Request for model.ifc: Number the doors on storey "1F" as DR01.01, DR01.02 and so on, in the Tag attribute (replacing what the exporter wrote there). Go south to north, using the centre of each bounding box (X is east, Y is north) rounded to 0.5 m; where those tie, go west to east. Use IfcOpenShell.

First a look at what the model holds.

```python
import ifcopenshell
import ifcopenshell.util.element
import ifcopenshell.util.placement

model = ifcopenshell.open("model.ifc")
print(model.schema)
storey = next(s for s in model.by_type("IfcBuildingStorey") if s.Name == "1F")
doors = [e for e in ifcopenshell.util.element.get_decomposition(storey) if e.is_a("IfcDoor")]
for e in sorted(doors, key=lambda e: e.id()):
    origin = ifcopenshell.util.placement.get_local_placement(e.ObjectPlacement)[:3, 3]
    print(e.id(), e.Tag, e.Name, origin.round(2) + 0.0, sep=" | ")
```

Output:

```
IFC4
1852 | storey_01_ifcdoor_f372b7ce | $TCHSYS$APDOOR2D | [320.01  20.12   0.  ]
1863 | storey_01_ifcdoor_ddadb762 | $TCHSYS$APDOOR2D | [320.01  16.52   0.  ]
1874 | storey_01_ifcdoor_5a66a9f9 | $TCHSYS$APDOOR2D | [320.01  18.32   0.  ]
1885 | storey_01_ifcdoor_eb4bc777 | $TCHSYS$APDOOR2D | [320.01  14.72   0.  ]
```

```python
import ifcopenshell
import ifcopenshell.geom
import ifcopenshell.util.element
import ifcopenshell.util.shape

model = ifcopenshell.open("model.ifc")
settings = ifcopenshell.geom.settings()
settings.set("use-world-coords", True)


def centre(element):
    shape = ifcopenshell.geom.create_shape(settings, element)
    return ifcopenshell.util.shape.get_bbox_centroid(shape.geometry)


storey = next(s for s in model.by_type("IfcBuildingStorey") if s.Name == "1F")
doors = [e for e in ifcopenshell.util.element.get_decomposition(storey) if e.is_a("IfcDoor")]

# Insertion points can sit at a corner or the storey origin, so sort by the geometry (in metres).
centres = {e: centre(e) for e in doors}
doors.sort(key=lambda e: (round(centres[e][1] / 0.5), centres[e][0]))

for i, e in enumerate(doors, start=1):
    number = f"DR01.{i:02d}"
    e.Tag = number
    print(e.id(), number)

model.write("model_rev.ifc")
```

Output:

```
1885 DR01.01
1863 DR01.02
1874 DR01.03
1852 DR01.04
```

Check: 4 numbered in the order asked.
